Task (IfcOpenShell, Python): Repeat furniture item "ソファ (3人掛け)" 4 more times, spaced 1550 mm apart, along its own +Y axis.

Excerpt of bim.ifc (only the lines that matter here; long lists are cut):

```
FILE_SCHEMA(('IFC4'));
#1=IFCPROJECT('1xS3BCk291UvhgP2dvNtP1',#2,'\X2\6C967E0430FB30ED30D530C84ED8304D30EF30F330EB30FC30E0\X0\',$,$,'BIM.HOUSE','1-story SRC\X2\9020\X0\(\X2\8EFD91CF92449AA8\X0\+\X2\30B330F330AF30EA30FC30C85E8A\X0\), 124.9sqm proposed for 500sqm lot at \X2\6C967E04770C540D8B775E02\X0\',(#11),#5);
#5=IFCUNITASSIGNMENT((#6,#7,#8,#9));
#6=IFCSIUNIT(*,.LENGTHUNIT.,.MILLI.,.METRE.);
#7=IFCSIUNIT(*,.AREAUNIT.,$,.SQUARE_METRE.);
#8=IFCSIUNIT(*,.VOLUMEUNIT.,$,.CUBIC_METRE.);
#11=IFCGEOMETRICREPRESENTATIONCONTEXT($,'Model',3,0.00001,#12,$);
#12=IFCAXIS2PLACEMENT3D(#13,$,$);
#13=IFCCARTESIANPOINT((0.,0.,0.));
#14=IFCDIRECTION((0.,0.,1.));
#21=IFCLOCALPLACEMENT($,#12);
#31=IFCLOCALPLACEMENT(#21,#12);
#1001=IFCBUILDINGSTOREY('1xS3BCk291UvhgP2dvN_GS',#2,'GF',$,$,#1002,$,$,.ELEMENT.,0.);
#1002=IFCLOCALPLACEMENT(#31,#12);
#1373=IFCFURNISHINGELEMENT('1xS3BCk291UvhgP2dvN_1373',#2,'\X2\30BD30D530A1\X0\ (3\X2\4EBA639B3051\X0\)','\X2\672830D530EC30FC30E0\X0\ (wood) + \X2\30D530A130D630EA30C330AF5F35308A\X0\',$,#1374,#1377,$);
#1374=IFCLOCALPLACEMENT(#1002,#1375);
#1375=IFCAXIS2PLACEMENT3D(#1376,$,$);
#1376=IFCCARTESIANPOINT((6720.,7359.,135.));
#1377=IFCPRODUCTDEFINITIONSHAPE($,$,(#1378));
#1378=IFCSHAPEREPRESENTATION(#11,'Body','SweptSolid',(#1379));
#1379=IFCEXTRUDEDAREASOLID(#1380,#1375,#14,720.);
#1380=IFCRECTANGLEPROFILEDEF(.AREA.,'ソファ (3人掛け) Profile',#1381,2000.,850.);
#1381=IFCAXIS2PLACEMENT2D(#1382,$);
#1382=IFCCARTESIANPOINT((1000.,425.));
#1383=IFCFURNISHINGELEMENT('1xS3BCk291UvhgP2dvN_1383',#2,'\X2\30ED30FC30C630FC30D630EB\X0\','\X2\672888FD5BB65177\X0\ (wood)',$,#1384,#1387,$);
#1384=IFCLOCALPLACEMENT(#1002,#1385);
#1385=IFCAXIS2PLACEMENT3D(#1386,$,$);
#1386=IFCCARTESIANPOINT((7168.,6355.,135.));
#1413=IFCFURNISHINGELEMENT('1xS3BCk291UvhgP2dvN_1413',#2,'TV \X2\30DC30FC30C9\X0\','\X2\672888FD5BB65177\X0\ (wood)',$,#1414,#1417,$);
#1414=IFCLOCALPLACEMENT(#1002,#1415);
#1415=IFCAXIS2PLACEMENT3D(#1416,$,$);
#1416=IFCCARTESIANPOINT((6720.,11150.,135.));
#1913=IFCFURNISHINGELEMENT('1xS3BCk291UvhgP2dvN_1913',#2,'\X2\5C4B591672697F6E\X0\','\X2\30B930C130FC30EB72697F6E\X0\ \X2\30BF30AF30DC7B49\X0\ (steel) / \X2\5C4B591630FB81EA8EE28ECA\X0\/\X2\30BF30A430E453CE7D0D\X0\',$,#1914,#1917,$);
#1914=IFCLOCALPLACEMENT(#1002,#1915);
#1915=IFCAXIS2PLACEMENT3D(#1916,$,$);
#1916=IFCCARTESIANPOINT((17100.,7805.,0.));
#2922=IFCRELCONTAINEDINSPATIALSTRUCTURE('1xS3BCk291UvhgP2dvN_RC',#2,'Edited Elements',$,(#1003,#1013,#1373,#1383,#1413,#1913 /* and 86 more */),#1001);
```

```python
import ifcopenshell
import ifcopenshell.api.geometry
import ifcopenshell.api.root
import ifcopenshell.util.element
import ifcopenshell.util.placement
import ifcopenshell.util.unit

model = ifcopenshell.open("bim.ifc")
unit_scale = ifcopenshell.util.unit.calculate_unit_scale(model)


def reuse_history(source, copy):
    """copy_class also copies each property set's owner history, people and application; keep the originals."""
    for rel in copy.IsDefinedBy:
        if rel.is_a("IfcRelDefinesByProperties") and (history := rel.RelatingPropertyDefinition.OwnerHistory):
            rel.RelatingPropertyDefinition.OwnerHistory = source.OwnerHistory
            ifcopenshell.util.element.remove_deep2(model, history)


source = model.by_id(1373)
base = ifcopenshell.util.placement.get_local_placement(source.ObjectPlacement)
step = base[:3, 1] * 1.55 / unit_scale

for i in range(1, 5):
    copy = ifcopenshell.api.root.copy_class(model, product=source)
    copy.Representation = ifcopenshell.util.element.copy_deep(
        model, source.Representation, exclude=["IfcGeometricRepresentationContext", "IfcRepresentationMap"]
    )
    reuse_history(source, copy)
    matrix = base.copy()
    matrix[:3, 3] += i * step
    print("added at", matrix[:3, 3].round(3) + 0.0)
    ifcopenshell.api.geometry.edit_object_placement(model, product=copy, matrix=matrix, is_si=False)

model.write("bim_v2.ifc")
```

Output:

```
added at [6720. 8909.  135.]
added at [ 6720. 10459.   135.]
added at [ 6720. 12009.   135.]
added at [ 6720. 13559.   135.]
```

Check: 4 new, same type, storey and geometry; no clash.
